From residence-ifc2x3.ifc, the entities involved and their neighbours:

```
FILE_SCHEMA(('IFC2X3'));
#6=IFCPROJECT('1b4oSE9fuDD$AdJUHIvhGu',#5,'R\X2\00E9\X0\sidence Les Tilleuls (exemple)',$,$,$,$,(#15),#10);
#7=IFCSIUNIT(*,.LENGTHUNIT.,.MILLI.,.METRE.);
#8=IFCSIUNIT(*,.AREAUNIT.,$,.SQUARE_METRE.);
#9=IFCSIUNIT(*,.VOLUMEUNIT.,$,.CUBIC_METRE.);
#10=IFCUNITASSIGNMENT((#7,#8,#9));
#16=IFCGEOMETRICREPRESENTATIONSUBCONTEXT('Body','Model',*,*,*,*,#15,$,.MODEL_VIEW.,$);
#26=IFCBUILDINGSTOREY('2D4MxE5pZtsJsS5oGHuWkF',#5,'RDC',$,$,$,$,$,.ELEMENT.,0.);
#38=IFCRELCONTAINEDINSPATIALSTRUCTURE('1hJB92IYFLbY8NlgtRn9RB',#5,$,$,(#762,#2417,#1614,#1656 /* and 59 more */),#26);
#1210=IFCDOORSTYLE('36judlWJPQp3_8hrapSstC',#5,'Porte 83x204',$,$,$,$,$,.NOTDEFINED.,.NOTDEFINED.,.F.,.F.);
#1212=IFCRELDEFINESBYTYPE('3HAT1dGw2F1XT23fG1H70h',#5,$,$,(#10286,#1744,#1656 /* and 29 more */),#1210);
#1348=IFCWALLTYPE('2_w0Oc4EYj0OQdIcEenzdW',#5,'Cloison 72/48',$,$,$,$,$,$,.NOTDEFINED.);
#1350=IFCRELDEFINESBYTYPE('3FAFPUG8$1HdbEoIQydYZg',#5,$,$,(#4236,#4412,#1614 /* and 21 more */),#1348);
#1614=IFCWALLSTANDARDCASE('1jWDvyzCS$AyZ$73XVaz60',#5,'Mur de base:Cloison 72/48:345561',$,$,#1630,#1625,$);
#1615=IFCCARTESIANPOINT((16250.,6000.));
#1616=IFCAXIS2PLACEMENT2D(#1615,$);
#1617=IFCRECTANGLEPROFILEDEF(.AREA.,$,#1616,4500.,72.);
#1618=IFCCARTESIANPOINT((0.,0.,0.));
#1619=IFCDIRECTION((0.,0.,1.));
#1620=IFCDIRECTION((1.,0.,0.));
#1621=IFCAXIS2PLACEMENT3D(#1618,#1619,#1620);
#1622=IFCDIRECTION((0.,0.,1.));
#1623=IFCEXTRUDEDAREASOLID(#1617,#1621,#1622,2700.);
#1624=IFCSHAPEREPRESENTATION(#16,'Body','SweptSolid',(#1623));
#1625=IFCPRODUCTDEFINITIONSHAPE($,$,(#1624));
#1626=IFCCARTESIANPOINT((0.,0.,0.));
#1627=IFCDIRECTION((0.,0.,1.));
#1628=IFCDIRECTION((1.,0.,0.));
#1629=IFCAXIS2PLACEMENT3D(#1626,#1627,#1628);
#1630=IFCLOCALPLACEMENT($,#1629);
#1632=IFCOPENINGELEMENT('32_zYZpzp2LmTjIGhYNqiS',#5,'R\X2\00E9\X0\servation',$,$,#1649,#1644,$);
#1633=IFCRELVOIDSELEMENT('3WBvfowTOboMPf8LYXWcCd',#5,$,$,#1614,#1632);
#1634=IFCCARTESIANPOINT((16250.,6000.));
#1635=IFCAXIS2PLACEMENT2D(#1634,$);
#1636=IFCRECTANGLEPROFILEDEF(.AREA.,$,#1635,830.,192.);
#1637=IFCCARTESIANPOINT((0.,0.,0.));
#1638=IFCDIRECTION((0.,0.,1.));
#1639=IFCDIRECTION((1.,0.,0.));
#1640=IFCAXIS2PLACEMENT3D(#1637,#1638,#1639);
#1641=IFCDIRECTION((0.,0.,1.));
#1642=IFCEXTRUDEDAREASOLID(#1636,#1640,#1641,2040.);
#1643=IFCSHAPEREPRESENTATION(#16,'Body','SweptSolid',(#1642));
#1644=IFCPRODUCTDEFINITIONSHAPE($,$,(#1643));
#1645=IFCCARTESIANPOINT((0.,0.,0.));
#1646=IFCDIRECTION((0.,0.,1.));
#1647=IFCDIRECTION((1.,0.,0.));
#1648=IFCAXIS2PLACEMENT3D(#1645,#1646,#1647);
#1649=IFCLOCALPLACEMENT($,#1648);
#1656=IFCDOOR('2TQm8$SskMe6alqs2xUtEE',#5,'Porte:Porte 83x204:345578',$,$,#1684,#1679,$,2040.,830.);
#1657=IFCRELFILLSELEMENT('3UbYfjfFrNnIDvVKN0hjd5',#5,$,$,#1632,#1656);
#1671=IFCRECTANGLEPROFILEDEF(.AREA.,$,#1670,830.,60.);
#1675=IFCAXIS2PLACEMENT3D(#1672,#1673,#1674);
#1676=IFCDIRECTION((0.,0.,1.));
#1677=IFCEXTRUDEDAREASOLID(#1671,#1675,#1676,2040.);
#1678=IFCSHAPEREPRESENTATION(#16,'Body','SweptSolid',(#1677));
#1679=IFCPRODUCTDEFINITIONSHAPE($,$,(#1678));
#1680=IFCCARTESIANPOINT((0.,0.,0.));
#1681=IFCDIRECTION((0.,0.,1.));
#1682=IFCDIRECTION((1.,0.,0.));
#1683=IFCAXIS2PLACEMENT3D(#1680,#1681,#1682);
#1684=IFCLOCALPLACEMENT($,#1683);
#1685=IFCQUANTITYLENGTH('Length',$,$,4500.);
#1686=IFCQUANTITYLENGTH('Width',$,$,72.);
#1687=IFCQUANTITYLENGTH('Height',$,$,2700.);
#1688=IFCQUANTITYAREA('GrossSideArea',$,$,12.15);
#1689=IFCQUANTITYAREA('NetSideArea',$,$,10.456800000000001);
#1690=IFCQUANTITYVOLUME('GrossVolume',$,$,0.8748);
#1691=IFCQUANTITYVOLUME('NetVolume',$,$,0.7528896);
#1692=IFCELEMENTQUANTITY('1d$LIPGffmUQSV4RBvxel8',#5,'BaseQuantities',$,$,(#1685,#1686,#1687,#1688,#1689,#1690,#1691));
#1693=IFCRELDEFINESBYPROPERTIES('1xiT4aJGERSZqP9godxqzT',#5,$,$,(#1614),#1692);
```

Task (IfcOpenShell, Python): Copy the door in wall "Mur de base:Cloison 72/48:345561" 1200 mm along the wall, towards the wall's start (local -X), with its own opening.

```python
import ifcopenshell
import ifcopenshell.api.feature
import ifcopenshell.api.geometry
import ifcopenshell.api.pset
import ifcopenshell.api.root
import ifcopenshell.geom
import ifcopenshell.util.element
import ifcopenshell.util.placement
import ifcopenshell.util.shape
import ifcopenshell.util.unit

model = ifcopenshell.open("residence-ifc2x3.ifc")
area_scale = ifcopenshell.util.unit.calculate_unit_scale(model, "AREAUNIT")
volume_scale = ifcopenshell.util.unit.calculate_unit_scale(model, "VOLUMEUNIT")
settings = ifcopenshell.geom.settings()


def volume(element):
    """Net volume in cubic metres, openings subtracted."""
    shape = ifcopenshell.geom.create_shape(settings, element)
    return ifcopenshell.util.shape.get_volume(shape.geometry)


def reuse_history(source, copy):
    """copy_class also copies each property set's owner history, people and application; keep the originals."""
    for rel in copy.IsDefinedBy:
        if rel.is_a("IfcRelDefinesByProperties") and (history := rel.RelatingPropertyDefinition.OwnerHistory):
            rel.RelatingPropertyDefinition.OwnerHistory = source.OwnerHistory
            ifcopenshell.util.element.remove_deep2(model, history)


door = model.by_guid("2TQm8$SskMe6alqs2xUtEE")
opening = door.FillsVoids[0].RelatingOpeningElement
wall = opening.VoidsElements[0].RelatingBuildingElement
before = volume(wall)
shift = ifcopenshell.util.placement.get_local_placement(wall.ObjectPlacement)[:3, 0] * -1200.0

# copy_class copies the void relationship, type, container and properties, but no geometry.
new_opening = ifcopenshell.api.root.copy_class(model, product=opening)
new_opening.Representation = ifcopenshell.util.element.copy_deep(
    model, opening.Representation, exclude=["IfcGeometricRepresentationContext", "IfcRepresentationMap"]
)
reuse_history(opening, new_opening)
new_door = ifcopenshell.api.root.copy_class(model, product=door)
new_door.Representation = ifcopenshell.util.element.copy_deep(
    model, door.Representation, exclude=["IfcGeometricRepresentationContext", "IfcRepresentationMap"]
)
new_door.Name = "Porte:Porte 83x204"
reuse_history(door, new_door)
fills = ifcopenshell.api.feature.add_filling(model, opening=new_opening, element=new_door)
fills.OwnerHistory = new_door.OwnerHistory  # required in IFC2X3

for old, new in ((opening, new_opening), (door, new_door)):
    matrix = ifcopenshell.util.placement.get_local_placement(old.ObjectPlacement)
    matrix[:3, 3] += shift
    ifcopenshell.api.geometry.edit_object_placement(model, product=new, matrix=matrix, is_si=False)

after = volume(wall)
thickness = 0.072  # wall thickness in metres

# Update the wall's stored quantities.
qto = model.by_id(ifcopenshell.util.element.get_pset(wall, "BaseQuantities", should_inherit=False)["id"])
ifcopenshell.api.pset.edit_qto(model, qto=qto, properties={
    "NetSideArea": after / thickness / area_scale,
    "NetVolume": after / volume_scale,
})

print(f"wall volume {before:.3f} -> {after:.3f} m3")

model.write("residence-ifc2x3-out.ifc")
```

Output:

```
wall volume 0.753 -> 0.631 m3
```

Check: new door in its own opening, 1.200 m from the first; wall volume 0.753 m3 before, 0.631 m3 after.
